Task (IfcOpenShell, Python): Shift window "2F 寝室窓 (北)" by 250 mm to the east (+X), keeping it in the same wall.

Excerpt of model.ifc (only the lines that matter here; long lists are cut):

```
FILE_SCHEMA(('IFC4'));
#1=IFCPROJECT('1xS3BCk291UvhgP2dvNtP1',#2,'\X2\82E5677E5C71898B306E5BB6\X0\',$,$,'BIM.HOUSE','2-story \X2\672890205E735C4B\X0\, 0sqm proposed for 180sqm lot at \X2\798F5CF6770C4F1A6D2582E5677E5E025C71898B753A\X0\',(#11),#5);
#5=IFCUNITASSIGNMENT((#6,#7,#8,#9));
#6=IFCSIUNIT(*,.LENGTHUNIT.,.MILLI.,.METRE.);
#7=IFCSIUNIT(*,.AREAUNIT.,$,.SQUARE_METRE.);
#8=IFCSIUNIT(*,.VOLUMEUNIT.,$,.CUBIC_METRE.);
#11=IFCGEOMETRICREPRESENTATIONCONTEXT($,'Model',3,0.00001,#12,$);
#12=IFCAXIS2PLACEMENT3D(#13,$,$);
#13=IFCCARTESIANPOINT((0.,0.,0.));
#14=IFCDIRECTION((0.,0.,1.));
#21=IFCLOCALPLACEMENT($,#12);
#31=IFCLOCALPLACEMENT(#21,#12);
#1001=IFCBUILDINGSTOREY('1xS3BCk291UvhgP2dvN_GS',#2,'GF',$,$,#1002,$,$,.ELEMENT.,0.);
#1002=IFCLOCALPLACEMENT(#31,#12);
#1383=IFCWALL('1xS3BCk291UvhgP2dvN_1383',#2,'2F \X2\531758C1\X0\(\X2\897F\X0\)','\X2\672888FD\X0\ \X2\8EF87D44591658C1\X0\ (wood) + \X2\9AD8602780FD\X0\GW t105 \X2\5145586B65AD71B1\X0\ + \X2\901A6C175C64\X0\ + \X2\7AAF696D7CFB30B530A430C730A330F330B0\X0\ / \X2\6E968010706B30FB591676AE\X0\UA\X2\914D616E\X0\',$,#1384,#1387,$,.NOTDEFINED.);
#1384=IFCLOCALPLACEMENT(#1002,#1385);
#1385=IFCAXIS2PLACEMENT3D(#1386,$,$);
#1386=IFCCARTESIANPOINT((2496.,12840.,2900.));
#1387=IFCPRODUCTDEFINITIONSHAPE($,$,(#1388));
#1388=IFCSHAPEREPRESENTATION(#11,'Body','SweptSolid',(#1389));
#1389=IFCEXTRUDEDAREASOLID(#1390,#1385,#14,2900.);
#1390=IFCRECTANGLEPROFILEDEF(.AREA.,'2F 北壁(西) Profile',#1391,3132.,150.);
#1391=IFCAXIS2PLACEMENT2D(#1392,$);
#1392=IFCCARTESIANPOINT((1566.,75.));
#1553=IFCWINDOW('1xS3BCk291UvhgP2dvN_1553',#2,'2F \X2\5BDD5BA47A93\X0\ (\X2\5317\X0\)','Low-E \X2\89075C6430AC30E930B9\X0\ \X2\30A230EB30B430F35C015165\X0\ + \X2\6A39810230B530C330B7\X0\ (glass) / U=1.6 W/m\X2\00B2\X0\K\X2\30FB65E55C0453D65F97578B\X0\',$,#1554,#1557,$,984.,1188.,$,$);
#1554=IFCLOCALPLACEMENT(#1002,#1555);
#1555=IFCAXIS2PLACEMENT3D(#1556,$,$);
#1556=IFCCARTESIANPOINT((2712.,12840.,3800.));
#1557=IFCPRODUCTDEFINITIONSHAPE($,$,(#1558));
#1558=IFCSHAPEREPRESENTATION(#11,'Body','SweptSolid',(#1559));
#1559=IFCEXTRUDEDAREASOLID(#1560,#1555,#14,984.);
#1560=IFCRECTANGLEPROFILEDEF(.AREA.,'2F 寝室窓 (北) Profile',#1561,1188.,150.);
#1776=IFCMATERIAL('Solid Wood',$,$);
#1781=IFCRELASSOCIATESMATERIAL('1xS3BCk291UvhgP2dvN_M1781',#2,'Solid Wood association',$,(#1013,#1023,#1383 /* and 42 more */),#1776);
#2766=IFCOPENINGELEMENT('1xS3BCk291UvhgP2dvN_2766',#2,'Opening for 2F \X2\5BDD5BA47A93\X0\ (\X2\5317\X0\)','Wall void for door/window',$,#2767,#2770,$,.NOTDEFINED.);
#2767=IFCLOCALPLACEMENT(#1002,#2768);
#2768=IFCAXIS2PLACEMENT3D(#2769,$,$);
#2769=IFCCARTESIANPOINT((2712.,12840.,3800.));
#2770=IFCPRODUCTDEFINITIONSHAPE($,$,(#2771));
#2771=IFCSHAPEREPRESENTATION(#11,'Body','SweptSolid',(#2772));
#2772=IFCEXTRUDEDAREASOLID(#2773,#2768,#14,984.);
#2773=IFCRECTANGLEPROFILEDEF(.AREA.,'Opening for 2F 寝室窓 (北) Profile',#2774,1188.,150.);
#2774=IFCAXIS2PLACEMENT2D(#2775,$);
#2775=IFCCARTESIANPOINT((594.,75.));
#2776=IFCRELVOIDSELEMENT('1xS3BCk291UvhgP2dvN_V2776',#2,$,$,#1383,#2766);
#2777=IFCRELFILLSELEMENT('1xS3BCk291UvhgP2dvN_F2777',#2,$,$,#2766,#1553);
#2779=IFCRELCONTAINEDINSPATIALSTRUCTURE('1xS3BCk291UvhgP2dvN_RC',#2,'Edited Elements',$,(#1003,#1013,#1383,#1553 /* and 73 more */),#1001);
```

```python
import ifcopenshell
import ifcopenshell.api.geometry
import ifcopenshell.util.placement
import ifcopenshell.util.unit

model = ifcopenshell.open("model.ifc")
unit_scale = ifcopenshell.util.unit.calculate_unit_scale(model)

window = model.by_guid("1xS3BCk291UvhgP2dvN_1553")
opening = window.FillsVoids[0].RelatingOpeningElement
wall = opening.VoidsElements[0].RelatingBuildingElement

wall_matrix = ifcopenshell.util.placement.get_local_placement(wall.ObjectPlacement)
shift = wall_matrix[:3, 0] * 0.25 / unit_scale
before = ifcopenshell.util.placement.get_local_placement(window.ObjectPlacement)[:3, 3].copy()

# The window is not placed relative to its opening, so move both.
for product in (opening, window):
    matrix = ifcopenshell.util.placement.get_local_placement(product.ObjectPlacement)
    matrix[:3, 3] += shift
    ifcopenshell.api.geometry.edit_object_placement(model, product=product, matrix=matrix, is_si=False)

after = ifcopenshell.util.placement.get_local_placement(window.ObjectPlacement)[:3, 3]
print("window moved by", (after - before).round(3) + 0.0)

model.write("model_v2.ifc")
```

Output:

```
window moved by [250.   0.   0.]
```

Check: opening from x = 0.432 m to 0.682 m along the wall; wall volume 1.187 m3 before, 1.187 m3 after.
